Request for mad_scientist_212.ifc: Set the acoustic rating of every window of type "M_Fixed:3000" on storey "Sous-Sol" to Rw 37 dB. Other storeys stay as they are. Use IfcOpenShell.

First a look at what the model holds.

```python
import ifcopenshell
import ifcopenshell.util.element

model = ifcopenshell.open("mad_scientist_212.ifc")
print(model.schema)
storey = next(s for s in model.by_type("IfcBuildingStorey") if s.Name == "Sous-Sol")
windows = [e for e in ifcopenshell.util.element.get_decomposition(storey) if e.is_a("IfcWindow")]
seen = {}
for e in windows:
    element_type = ifcopenshell.util.element.get_type(e)
    key = (element_type.Name if element_type != e and element_type else None, ifcopenshell.util.element.get_pset(e, "Pset_WindowCommon", "AcousticRating"))
    seen[key] = seen.get(key, 0) + 1
for (name, value), count in sorted(seen.items(), key=str):
    print(count, "x", name, "|", value)
```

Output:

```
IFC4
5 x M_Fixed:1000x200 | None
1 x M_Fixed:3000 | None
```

```python
import ifcopenshell
import ifcopenshell.api.pset
import ifcopenshell.util.element

model = ifcopenshell.open("mad_scientist_212.ifc")

storey = next(s for s in model.by_type("IfcBuildingStorey") if s.Name == "Sous-Sol")
windows = [e for e in ifcopenshell.util.element.get_decomposition(storey) if e.is_a("IfcWindow")]

count = 0
for e in windows:
    element_type = ifcopenshell.util.element.get_type(e)
    if element_type in (None, e) or element_type.Name != "M_Fixed:3000":
        continue
    # add_pset returns the element's existing set when there is one.
    pset = ifcopenshell.api.pset.add_pset(model, product=e, name="Pset_WindowCommon")
    ifcopenshell.api.pset.edit_pset(model, pset=pset, properties={"AcousticRating": "Rw 37 dB"})
    count += 1

print(count, "windows updated")

model.write("mad_scientist_212-out.ifc")
```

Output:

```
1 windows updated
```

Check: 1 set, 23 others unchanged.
